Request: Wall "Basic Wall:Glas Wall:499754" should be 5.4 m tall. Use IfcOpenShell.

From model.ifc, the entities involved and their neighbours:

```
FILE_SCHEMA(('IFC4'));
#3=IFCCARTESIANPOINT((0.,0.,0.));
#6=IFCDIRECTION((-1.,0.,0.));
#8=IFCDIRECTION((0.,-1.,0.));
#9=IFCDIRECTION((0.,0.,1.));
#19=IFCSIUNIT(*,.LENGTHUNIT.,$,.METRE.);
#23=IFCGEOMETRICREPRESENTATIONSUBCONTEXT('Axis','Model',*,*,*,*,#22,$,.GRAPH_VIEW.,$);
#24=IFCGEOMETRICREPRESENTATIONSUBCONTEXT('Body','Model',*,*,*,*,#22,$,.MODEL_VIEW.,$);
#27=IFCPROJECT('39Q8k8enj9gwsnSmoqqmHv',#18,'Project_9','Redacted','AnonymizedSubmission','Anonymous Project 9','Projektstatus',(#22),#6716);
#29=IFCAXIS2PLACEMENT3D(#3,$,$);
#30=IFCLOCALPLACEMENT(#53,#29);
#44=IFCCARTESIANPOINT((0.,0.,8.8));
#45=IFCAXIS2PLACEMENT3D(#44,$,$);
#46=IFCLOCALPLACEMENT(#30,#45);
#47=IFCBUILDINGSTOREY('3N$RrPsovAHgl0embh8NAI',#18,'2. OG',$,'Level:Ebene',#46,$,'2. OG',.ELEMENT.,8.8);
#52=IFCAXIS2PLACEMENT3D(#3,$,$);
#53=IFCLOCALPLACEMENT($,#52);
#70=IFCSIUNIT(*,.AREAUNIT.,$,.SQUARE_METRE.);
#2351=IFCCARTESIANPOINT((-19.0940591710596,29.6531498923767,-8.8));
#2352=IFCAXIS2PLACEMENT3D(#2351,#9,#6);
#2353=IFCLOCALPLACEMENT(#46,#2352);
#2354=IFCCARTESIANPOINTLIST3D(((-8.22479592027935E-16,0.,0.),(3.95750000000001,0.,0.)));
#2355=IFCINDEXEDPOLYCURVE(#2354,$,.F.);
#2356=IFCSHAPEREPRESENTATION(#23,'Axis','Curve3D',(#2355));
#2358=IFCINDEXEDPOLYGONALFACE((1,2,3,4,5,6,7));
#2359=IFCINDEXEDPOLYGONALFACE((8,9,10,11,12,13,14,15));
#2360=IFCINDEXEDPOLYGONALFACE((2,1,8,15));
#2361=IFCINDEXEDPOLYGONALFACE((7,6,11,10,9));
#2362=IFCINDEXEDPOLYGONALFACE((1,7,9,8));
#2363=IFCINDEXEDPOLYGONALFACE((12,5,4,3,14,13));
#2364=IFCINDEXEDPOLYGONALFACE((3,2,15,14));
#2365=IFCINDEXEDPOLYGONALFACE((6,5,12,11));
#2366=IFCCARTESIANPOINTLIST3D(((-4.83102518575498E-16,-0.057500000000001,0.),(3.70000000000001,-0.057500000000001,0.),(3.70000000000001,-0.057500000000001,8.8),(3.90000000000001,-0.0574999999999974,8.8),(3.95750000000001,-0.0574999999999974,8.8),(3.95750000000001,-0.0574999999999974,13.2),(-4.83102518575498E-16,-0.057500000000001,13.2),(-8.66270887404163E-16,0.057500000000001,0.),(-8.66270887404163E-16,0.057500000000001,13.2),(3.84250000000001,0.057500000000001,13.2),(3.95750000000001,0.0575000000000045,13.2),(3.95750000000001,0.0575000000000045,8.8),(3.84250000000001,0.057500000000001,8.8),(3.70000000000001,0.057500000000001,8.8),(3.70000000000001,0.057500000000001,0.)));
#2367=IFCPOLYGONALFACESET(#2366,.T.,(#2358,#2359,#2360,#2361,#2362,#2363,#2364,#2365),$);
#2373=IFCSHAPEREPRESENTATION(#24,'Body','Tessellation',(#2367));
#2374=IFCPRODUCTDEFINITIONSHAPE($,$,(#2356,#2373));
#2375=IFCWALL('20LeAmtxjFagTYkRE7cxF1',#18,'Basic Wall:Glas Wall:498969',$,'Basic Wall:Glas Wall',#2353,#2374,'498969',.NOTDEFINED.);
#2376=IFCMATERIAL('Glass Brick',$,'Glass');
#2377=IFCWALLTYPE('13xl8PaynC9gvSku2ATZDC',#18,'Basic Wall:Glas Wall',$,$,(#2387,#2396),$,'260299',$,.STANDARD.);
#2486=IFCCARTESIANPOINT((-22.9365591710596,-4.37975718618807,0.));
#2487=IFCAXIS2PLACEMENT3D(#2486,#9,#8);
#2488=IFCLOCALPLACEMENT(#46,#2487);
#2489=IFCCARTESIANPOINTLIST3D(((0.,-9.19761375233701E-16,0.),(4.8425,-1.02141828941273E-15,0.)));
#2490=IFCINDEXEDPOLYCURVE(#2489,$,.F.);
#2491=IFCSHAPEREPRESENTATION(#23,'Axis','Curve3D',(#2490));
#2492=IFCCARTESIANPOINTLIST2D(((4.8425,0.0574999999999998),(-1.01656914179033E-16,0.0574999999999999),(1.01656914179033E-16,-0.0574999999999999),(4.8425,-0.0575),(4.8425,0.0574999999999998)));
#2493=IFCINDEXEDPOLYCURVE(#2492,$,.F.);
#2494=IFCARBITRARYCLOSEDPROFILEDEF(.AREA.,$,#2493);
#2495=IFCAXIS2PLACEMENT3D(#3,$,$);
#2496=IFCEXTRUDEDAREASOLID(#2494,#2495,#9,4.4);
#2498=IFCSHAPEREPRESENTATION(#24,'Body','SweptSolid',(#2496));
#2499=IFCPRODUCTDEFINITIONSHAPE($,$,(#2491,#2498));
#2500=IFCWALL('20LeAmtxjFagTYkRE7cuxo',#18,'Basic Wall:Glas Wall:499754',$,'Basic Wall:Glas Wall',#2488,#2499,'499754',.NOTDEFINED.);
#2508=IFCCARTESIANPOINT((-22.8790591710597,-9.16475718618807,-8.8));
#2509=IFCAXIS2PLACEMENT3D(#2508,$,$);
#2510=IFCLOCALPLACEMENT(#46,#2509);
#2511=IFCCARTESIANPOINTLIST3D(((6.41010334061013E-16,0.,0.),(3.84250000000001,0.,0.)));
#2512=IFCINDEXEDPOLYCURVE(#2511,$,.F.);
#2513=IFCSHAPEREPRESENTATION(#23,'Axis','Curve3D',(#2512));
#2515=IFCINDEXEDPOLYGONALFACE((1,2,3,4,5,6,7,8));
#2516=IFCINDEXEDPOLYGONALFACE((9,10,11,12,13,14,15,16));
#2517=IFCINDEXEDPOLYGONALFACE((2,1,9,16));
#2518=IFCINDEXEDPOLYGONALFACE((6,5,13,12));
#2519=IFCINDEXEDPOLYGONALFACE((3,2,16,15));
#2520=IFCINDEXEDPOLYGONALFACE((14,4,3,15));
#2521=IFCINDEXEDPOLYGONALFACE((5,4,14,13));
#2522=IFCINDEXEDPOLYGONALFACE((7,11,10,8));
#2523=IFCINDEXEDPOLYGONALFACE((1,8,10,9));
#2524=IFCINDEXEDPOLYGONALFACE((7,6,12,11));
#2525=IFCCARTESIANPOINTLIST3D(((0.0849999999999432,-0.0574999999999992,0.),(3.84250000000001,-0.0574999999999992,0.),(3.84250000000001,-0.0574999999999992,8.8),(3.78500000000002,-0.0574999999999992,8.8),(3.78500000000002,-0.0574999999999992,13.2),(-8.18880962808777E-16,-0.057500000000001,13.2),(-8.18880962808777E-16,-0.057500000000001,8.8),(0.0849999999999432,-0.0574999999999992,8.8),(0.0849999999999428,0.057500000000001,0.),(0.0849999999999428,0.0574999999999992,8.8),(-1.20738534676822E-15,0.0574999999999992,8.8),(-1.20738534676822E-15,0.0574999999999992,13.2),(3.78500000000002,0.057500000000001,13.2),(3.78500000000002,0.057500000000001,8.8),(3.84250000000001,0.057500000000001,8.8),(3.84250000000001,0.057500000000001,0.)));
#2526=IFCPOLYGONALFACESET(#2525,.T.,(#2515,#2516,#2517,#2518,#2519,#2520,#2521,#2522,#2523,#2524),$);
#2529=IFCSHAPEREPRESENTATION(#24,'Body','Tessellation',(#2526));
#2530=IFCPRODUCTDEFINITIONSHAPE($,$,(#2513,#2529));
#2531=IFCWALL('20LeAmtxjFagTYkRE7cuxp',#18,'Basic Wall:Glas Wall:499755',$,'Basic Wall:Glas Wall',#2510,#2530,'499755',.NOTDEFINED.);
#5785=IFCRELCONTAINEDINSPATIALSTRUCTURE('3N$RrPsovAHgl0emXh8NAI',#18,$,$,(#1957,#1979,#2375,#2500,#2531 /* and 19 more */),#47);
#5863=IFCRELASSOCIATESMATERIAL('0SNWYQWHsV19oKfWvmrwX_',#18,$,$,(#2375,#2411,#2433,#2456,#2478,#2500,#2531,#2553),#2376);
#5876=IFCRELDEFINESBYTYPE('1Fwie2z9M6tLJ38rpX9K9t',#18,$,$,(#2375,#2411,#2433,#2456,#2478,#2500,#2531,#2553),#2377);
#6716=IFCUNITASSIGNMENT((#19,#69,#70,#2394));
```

```python
import ifcopenshell
import ifcopenshell.geom
import ifcopenshell.util.representation
import ifcopenshell.util.shape

model = ifcopenshell.open("model.ifc")
settings = ifcopenshell.geom.settings()


def volume(element):
    """Net volume in cubic metres, openings subtracted."""
    shape = ifcopenshell.geom.create_shape(settings, element)
    return ifcopenshell.util.shape.get_volume(shape.geometry)


wall = model.by_id(2500)
before = volume(wall)

body = ifcopenshell.util.representation.get_representation(wall, "Model", "Body")
solid = body.Items[0]
old_height = solid.Depth
solid.Depth = 5.4
after = volume(wall)

print(f"height {old_height:g} -> {solid.Depth:g}, volume {before:.3f} -> {after:.3f} m3")

model.write("model_rev.ifc")
```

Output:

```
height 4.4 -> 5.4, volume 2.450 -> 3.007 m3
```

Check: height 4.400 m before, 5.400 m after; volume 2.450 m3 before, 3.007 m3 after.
